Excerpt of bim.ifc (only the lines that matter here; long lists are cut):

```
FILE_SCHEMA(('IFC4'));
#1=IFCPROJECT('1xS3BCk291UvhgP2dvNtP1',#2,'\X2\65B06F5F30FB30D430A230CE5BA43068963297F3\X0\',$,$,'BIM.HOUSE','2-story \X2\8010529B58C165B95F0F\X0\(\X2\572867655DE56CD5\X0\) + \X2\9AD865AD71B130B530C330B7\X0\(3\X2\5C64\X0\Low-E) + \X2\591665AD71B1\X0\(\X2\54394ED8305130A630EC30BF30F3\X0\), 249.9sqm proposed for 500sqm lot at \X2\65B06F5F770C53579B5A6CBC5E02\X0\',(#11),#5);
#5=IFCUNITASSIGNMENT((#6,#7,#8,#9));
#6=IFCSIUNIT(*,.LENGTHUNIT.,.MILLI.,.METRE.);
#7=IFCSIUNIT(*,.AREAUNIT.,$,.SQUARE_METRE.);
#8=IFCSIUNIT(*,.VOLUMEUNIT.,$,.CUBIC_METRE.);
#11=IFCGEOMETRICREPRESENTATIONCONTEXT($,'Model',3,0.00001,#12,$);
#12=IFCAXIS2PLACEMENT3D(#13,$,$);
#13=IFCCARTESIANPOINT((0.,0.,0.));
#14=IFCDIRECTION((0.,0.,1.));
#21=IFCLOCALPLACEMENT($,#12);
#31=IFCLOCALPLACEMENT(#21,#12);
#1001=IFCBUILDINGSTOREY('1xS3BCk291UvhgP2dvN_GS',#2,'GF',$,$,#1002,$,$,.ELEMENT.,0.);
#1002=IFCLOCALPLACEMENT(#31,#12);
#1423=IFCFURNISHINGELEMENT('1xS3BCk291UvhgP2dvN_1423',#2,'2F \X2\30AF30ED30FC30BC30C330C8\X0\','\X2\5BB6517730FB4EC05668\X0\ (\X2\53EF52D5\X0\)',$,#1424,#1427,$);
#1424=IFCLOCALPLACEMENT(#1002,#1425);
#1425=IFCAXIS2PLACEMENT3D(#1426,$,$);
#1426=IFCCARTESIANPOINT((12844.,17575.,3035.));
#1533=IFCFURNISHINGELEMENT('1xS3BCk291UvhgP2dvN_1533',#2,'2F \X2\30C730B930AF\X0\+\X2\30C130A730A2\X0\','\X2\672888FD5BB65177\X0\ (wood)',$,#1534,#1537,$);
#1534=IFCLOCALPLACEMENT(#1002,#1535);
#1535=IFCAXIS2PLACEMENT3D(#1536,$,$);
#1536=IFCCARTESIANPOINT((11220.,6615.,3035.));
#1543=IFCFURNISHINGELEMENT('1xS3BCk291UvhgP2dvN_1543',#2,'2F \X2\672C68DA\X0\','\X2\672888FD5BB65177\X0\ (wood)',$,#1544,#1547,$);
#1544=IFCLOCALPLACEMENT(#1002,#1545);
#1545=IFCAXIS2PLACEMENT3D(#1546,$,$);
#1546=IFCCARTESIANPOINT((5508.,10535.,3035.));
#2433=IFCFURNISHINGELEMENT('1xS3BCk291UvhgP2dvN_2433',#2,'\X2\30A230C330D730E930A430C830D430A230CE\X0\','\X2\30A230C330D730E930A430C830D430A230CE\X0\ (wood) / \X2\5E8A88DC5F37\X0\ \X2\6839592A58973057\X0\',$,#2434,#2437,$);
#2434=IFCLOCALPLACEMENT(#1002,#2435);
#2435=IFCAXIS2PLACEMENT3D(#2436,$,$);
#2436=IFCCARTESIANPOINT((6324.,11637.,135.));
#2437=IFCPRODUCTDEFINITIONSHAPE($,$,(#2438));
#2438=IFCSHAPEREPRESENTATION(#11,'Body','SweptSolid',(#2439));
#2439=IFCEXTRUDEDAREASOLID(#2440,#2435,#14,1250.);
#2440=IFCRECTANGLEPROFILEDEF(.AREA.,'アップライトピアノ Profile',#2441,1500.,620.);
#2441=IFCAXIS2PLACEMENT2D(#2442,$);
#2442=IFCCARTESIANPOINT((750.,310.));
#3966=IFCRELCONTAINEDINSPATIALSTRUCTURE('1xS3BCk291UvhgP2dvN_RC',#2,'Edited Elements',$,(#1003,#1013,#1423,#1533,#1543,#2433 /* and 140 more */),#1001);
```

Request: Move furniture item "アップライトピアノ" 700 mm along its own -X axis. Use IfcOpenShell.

```python
import ifcopenshell
import ifcopenshell.api.geometry
import ifcopenshell.util.placement
import ifcopenshell.util.unit

model = ifcopenshell.open("bim.ifc")
unit_scale = ifcopenshell.util.unit.calculate_unit_scale(model)

item = model.by_id(2433)
matrix = ifcopenshell.util.placement.get_local_placement(item.ObjectPlacement)
matrix[:3, 3] -= matrix[:3, 0] * 0.7 / unit_scale
ifcopenshell.api.geometry.edit_object_placement(model, product=item, matrix=matrix, is_si=False)

print(ifcopenshell.util.placement.get_local_placement(item.ObjectPlacement).round(3) + 0.0)

model.write("bim_edited.ifc")
```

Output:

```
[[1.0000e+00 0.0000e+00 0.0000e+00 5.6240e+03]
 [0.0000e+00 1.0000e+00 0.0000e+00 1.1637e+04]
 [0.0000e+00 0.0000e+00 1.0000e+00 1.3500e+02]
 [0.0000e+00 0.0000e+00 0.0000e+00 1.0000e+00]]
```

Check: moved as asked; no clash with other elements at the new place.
